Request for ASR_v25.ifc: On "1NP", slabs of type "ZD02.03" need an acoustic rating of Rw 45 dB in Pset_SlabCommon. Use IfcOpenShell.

First a look at what the model holds.

```python
import ifcopenshell
import ifcopenshell.util.element

model = ifcopenshell.open("ASR_v25.ifc")
print(model.schema)
storey = next(s for s in model.by_type("IfcBuildingStorey") if s.Name == "1NP")
slabs = [e for e in ifcopenshell.util.element.get_decomposition(storey) if e.is_a("IfcSlab")]
seen = {}
for e in slabs:
    element_type = ifcopenshell.util.element.get_type(e)
    key = (element_type.Name if element_type != e and element_type else None, ifcopenshell.util.element.get_pset(e, "Pset_SlabCommon", "AcousticRating"))
    seen[key] = seen.get(key, 0) + 1
for (name, value), count in sorted(seen.items(), key=str):
    print(count, "x", name, "|", value)
```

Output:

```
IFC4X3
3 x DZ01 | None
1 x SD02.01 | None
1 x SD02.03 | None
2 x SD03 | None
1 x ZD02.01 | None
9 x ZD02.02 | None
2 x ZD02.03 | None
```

```python
import ifcopenshell
import ifcopenshell.api.pset
import ifcopenshell.util.element

model = ifcopenshell.open("ASR_v25.ifc")

storey = next(s for s in model.by_type("IfcBuildingStorey") if s.Name == "1NP")
slabs = [e for e in ifcopenshell.util.element.get_decomposition(storey) if e.is_a("IfcSlab")]

count = 0
for e in slabs:
    element_type = ifcopenshell.util.element.get_type(e)
    if element_type in (None, e) or element_type.Name != "ZD02.03":
        continue
    # add_pset returns the element's existing set when there is one.
    pset = ifcopenshell.api.pset.add_pset(model, product=e, name="Pset_SlabCommon")
    ifcopenshell.api.pset.edit_pset(model, pset=pset, properties={"AcousticRating": "Rw 45 dB"})
    count += 1

print(count, "slabs updated")

model.write("ASR_v25_edited.ifc")
```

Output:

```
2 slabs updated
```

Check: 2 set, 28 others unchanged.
